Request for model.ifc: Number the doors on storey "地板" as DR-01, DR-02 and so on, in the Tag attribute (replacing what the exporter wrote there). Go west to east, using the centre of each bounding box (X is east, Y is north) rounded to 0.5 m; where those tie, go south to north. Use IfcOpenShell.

First a look at what the model holds.

```python
import ifcopenshell
import ifcopenshell.util.element
import ifcopenshell.util.placement

model = ifcopenshell.open("model.ifc")
print(model.schema)
storey = next(s for s in model.by_type("IfcBuildingStorey") if s.Name == "地板")
doors = [e for e in ifcopenshell.util.element.get_decomposition(storey) if e.is_a("IfcDoor")]
for e in sorted(doors, key=lambda e: e.id()):
    origin = ifcopenshell.util.placement.get_local_placement(e.ObjectPlacement)[:3, 3]
    print(e.id(), e.Tag, e.Name, origin.round(2) + 0.0, sep=" | ")
```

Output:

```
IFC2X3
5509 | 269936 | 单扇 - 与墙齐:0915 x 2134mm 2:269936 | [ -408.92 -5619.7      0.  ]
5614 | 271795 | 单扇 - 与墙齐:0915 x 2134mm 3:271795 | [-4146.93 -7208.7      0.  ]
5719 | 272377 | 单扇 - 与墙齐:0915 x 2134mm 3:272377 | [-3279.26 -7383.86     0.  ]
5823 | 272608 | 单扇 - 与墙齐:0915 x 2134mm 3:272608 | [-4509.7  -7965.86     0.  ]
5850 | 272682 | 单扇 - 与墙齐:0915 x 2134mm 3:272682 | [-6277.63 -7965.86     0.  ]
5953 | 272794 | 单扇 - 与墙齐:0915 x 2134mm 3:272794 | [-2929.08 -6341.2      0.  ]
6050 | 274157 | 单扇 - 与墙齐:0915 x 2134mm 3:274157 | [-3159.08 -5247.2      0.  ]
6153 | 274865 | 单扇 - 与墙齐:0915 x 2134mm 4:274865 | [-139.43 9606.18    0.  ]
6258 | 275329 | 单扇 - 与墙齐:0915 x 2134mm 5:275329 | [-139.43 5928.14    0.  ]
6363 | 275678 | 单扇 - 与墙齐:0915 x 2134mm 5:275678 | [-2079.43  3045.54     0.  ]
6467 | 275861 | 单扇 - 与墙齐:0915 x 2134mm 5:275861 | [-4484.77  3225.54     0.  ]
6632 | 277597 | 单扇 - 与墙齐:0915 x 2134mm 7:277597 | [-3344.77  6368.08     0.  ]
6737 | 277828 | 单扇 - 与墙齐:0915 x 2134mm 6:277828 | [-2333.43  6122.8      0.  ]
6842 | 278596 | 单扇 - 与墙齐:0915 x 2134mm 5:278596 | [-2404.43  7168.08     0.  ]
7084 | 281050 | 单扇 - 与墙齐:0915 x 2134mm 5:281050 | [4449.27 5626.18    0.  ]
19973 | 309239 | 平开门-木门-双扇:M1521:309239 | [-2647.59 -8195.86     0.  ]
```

```python
import ifcopenshell
import ifcopenshell.geom
import ifcopenshell.util.element
import ifcopenshell.util.shape

model = ifcopenshell.open("model.ifc")
settings = ifcopenshell.geom.settings()
settings.set("use-world-coords", True)


def centre(element):
    shape = ifcopenshell.geom.create_shape(settings, element)
    return ifcopenshell.util.shape.get_bbox_centroid(shape.geometry)


storey = next(s for s in model.by_type("IfcBuildingStorey") if s.Name == "地板")
doors = [e for e in ifcopenshell.util.element.get_decomposition(storey) if e.is_a("IfcDoor")]

# Insertion points can sit at a corner or the storey origin, so sort by the geometry (in metres).
centres = {e: centre(e) for e in doors}
doors.sort(key=lambda e: (round(centres[e][0] / 0.5), centres[e][1]))

for i, e in enumerate(doors, start=1):
    number = f"DR-{i:02d}"
    e.Tag = number
    print(e.id(), number)

model.write("model_rev.ifc")
```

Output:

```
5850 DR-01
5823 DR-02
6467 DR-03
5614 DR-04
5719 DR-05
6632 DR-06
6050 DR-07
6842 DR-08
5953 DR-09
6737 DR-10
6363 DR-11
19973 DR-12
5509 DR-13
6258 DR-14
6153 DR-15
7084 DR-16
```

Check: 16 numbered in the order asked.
